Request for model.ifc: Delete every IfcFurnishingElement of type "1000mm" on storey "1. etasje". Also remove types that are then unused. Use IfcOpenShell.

First a look at what the model holds.

```python
import ifcopenshell
import ifcopenshell.util.element

model = ifcopenshell.open("model.ifc")
print(model.schema)
storey = next(s for s in model.by_type("IfcBuildingStorey") if s.Name == "1. etasje")
furniture = [e for e in ifcopenshell.util.element.get_decomposition(storey) if e.is_a("IfcFurnishingElement")]
seen = {}
for e in furniture:
    element_type = ifcopenshell.util.element.get_type(e)
    name = element_type.Name if element_type not in (None, e) else None
    seen[name] = seen.get(name, 0) + 1
for name, count in sorted(seen.items(), key=str):
    print(count, "x", name)
```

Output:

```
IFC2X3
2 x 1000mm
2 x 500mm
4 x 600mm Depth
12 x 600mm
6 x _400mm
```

```python
import ifcopenshell
import ifcopenshell.api.root
import ifcopenshell.util.element

model = ifcopenshell.open("model.ifc")

storey = next(s for s in model.by_type("IfcBuildingStorey") if s.Name == "1. etasje")
furniture = [e for e in ifcopenshell.util.element.get_decomposition(storey) if e.is_a("IfcFurnishingElement")]
targets = [e for e in furniture if (t := ifcopenshell.util.element.get_type(e)) not in (None, e) and t.Name == "1000mm"]
types = {ifcopenshell.util.element.get_type(e) for e in targets} - {None, *targets}

for e in targets:
    ifcopenshell.api.root.remove_product(model, product=e)
print(len(targets), "removed")

unused = [t for t in types if not ifcopenshell.util.element.get_types(t)]
for t in unused:
    ifcopenshell.api.root.remove_product(model, product=t)
print(len(unused), "unused types removed")

model.write("model_updated.ifc")
```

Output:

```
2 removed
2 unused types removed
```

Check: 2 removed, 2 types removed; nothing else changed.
